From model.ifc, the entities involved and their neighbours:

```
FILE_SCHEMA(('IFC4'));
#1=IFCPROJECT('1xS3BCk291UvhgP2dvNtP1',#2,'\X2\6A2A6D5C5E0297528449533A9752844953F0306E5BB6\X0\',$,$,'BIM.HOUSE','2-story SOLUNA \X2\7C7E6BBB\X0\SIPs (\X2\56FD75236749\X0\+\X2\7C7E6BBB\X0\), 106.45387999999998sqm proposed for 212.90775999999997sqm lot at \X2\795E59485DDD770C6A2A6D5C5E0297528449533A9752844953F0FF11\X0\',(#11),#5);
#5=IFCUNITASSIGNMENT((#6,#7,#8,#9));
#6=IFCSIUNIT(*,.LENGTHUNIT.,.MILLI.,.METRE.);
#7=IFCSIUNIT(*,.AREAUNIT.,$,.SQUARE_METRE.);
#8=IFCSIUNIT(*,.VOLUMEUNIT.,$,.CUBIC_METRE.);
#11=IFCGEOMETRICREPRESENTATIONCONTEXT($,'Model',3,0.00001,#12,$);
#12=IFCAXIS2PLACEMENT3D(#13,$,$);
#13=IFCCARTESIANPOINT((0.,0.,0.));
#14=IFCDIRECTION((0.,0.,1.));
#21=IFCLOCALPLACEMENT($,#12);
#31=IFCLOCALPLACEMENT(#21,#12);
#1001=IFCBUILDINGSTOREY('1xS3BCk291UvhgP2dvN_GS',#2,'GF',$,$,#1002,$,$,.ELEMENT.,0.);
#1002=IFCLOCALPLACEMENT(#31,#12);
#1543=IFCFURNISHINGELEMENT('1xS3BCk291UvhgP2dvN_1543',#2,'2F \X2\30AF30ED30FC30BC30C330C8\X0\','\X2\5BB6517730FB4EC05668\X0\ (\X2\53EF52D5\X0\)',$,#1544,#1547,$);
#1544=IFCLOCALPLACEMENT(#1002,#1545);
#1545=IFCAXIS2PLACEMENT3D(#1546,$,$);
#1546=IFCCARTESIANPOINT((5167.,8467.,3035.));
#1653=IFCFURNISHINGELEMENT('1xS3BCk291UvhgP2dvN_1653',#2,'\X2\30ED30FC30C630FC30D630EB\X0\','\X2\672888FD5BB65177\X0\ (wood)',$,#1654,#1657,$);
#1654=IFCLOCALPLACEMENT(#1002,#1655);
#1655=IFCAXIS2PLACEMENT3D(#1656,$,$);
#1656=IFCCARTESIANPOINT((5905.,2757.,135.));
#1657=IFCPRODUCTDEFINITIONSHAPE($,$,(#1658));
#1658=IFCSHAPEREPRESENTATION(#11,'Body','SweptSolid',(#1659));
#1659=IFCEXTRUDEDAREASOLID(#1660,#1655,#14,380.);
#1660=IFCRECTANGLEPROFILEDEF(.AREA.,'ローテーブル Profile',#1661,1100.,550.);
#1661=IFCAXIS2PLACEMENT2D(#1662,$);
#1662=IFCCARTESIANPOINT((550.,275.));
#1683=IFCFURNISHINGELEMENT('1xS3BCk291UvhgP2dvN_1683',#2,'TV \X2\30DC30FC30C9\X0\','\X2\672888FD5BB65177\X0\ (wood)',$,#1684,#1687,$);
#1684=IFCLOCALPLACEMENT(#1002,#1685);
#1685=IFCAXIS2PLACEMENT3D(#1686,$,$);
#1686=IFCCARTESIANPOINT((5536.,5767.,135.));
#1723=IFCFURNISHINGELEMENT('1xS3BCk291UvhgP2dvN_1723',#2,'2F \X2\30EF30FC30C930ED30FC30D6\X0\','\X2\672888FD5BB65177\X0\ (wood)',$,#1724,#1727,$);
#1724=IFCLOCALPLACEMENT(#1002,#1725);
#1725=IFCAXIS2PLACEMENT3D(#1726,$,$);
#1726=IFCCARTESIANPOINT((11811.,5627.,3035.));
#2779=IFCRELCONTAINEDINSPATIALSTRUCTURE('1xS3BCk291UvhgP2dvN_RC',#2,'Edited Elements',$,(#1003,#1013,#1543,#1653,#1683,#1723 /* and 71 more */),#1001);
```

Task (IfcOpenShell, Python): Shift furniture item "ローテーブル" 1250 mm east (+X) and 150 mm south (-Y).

```python
import ifcopenshell
import ifcopenshell.api.geometry
import ifcopenshell.util.placement

model = ifcopenshell.open("model.ifc")

item = model.by_guid("1xS3BCk291UvhgP2dvN_1653")
matrix = ifcopenshell.util.placement.get_local_placement(item.ObjectPlacement)
matrix[0, 3] += 1250.0
matrix[1, 3] -= 150.0
ifcopenshell.api.geometry.edit_object_placement(model, product=item, matrix=matrix, is_si=False)

print(ifcopenshell.util.placement.get_local_placement(item.ObjectPlacement).round(3) + 0.0)

model.write("model_updated.ifc")
```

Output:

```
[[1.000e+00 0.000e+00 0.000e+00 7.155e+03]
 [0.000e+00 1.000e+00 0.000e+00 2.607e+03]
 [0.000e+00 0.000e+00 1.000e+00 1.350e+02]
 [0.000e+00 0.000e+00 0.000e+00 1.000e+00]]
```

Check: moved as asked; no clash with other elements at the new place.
